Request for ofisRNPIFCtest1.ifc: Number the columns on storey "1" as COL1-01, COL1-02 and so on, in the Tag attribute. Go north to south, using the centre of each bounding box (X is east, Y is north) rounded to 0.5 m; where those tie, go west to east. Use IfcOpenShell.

First a look at what the model holds.

```python
import ifcopenshell
import ifcopenshell.util.element
import ifcopenshell.util.placement

model = ifcopenshell.open("ofisRNPIFCtest1.ifc")
print(model.schema)
storey = next(s for s in model.by_type("IfcBuildingStorey") if s.Name == "1")
columns = [e for e in ifcopenshell.util.element.get_decomposition(storey) if e.is_a("IfcColumn")]
for e in sorted(columns, key=lambda e: e.id()):
    origin = ifcopenshell.util.placement.get_local_placement(e.ObjectPlacement)[:3, 3]
    print(e.id(), e.Tag, e.Name, origin.round(2) + 0.0, sep=" | ")
```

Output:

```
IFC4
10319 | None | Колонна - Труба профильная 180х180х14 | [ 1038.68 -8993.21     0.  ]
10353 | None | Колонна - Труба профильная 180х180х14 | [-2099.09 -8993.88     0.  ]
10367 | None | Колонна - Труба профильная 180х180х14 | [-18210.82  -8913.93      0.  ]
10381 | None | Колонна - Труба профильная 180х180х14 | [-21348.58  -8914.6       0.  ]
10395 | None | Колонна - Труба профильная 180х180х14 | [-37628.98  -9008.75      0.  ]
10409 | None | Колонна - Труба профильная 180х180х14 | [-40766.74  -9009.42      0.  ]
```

```python
import ifcopenshell
import ifcopenshell.geom
import ifcopenshell.util.element
import ifcopenshell.util.shape

model = ifcopenshell.open("ofisRNPIFCtest1.ifc")
settings = ifcopenshell.geom.settings()
settings.set("use-world-coords", True)


def centre(element):
    shape = ifcopenshell.geom.create_shape(settings, element)
    return ifcopenshell.util.shape.get_bbox_centroid(shape.geometry)


storey = next(s for s in model.by_type("IfcBuildingStorey") if s.Name == "1")
columns = [e for e in ifcopenshell.util.element.get_decomposition(storey) if e.is_a("IfcColumn")]

# Insertion points can sit at a corner or the storey origin, so sort by the geometry (in metres).
centres = {e: centre(e) for e in columns}
columns.sort(key=lambda e: (-round(centres[e][1] / 0.5), centres[e][0]))

for i, e in enumerate(columns, start=1):
    number = f"COL1-{i:02d}"
    e.Tag = number
    print(e.id(), number)

model.write("ofisRNPIFCtest1_edited.ifc")
```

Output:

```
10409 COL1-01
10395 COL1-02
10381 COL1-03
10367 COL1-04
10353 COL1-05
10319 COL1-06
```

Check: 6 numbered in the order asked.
